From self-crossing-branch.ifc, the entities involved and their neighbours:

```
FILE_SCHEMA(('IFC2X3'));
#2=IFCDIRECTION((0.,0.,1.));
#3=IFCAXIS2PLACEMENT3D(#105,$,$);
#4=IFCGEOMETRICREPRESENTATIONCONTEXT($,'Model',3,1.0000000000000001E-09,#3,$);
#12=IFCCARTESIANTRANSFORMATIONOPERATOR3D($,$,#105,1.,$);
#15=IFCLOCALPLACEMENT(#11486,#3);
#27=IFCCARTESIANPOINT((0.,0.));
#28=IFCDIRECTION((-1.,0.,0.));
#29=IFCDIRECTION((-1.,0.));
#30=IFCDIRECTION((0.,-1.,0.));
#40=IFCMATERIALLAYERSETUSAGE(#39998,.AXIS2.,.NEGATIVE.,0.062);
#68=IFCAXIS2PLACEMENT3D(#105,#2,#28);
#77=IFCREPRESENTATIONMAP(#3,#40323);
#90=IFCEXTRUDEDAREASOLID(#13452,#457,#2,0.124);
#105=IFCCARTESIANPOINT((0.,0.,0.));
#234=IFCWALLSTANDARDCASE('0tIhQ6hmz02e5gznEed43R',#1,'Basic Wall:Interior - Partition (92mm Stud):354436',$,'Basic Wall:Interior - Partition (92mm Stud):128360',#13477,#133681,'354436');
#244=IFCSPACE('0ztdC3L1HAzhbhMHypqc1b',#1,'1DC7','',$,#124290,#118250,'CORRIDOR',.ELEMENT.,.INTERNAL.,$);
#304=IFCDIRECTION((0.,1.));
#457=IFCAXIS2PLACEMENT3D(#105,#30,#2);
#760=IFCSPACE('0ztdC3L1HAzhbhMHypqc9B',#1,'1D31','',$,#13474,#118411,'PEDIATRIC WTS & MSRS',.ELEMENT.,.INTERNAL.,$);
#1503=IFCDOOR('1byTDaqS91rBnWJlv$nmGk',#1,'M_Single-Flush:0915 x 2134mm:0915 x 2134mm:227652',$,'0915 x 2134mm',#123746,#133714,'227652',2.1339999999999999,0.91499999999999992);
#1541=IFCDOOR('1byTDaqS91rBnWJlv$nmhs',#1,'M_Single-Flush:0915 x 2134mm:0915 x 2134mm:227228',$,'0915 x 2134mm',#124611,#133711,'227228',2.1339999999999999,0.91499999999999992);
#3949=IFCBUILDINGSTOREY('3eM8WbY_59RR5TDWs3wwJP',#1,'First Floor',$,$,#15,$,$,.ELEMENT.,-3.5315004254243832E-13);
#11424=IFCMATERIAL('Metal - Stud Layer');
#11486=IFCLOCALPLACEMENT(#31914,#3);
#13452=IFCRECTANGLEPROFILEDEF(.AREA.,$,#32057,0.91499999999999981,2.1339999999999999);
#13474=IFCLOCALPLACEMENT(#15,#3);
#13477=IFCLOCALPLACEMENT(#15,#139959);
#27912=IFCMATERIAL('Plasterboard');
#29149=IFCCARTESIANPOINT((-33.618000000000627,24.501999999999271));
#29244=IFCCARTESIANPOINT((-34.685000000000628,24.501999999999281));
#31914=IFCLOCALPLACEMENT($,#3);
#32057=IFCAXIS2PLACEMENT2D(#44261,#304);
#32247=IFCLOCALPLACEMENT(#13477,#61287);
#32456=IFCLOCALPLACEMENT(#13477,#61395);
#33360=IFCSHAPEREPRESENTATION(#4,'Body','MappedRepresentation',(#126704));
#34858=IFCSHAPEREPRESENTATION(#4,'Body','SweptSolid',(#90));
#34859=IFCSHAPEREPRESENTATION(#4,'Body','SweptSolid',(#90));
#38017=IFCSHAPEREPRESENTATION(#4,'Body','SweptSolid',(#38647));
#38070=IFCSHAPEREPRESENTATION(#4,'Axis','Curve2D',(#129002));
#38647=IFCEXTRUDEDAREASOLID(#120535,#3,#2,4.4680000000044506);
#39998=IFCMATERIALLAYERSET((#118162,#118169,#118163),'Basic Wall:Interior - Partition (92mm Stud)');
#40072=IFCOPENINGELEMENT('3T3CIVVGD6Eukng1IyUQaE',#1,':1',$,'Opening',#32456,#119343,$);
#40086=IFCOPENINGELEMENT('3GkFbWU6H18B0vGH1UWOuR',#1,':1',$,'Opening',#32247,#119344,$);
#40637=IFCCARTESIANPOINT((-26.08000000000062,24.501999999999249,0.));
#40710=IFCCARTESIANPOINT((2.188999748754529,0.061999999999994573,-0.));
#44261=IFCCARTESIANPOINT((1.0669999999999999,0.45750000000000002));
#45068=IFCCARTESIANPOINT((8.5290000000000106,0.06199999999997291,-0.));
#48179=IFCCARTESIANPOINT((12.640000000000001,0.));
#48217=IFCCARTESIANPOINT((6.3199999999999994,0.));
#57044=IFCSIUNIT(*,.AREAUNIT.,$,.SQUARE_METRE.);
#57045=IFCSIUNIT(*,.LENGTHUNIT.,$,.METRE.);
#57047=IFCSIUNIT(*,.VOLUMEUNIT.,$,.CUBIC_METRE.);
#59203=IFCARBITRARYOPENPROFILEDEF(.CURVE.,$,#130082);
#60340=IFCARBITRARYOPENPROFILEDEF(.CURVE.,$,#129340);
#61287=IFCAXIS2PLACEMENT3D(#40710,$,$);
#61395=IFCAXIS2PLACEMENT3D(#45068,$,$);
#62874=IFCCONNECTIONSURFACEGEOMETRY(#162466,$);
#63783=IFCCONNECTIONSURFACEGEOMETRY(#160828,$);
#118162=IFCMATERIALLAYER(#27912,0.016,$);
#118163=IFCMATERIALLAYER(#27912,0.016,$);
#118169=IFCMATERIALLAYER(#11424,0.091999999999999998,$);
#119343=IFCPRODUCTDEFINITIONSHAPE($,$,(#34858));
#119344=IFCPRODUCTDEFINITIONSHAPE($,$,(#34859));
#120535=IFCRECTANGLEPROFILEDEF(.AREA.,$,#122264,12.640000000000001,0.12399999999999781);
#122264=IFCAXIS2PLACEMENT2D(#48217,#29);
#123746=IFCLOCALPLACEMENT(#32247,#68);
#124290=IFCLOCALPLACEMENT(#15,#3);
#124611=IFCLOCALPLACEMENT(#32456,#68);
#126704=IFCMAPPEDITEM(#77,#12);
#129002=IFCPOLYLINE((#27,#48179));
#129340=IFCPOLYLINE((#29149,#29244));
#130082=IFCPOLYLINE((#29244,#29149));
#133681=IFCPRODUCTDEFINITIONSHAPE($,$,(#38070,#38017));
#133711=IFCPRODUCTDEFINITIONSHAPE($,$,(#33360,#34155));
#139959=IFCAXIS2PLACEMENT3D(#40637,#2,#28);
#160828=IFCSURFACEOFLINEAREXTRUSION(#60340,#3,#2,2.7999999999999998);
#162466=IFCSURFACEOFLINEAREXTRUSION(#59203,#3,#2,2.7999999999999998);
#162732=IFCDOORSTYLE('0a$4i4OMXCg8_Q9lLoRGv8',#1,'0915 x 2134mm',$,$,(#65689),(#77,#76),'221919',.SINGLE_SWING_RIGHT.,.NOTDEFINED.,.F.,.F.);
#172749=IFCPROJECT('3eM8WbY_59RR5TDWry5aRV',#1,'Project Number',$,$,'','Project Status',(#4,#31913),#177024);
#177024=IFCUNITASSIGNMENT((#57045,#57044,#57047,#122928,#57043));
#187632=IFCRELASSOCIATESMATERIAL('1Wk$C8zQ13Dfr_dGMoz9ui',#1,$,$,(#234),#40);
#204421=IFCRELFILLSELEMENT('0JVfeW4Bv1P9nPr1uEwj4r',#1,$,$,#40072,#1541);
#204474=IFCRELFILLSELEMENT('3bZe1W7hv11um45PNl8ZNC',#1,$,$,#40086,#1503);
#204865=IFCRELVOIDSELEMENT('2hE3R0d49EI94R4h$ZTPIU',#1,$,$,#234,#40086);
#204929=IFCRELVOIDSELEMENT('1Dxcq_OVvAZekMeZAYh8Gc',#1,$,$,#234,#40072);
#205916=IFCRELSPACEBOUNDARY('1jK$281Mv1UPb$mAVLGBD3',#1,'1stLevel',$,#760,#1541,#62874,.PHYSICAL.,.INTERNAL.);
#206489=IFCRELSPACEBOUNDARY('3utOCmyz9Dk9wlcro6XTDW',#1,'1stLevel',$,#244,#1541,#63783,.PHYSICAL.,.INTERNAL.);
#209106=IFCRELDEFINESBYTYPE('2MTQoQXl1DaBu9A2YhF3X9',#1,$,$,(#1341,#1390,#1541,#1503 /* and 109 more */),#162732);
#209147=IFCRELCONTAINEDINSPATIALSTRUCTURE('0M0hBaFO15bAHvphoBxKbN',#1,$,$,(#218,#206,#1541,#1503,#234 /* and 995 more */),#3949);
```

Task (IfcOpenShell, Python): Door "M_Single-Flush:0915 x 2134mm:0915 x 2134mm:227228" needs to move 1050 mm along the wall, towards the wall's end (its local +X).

```python
import numpy as np
import ifcopenshell
import ifcopenshell.api.geometry
import ifcopenshell.util.placement

model = ifcopenshell.open("self-crossing-branch.ifc")

door = model.by_id(1541)
opening = door.FillsVoids[0].RelatingOpeningElement
wall = opening.VoidsElements[0].RelatingBuildingElement

wall_matrix = ifcopenshell.util.placement.get_local_placement(wall.ObjectPlacement)
shift = wall_matrix[:3, 0] * 1.05
before = ifcopenshell.util.placement.get_local_placement(door.ObjectPlacement)[:3, 3].copy()

# The door is placed relative to its opening, so it follows when the opening moves.
matrix = ifcopenshell.util.placement.get_local_placement(opening.ObjectPlacement)
matrix[:3, 3] += shift
ifcopenshell.api.geometry.edit_object_placement(
    model, product=opening, matrix=matrix, is_si=False, should_transform_children=True
)

# Space boundary surfaces are stored in each space's coordinates; move them too.
for rel in door.ProvidesBoundaries:
    if not rel.ConnectionGeometry:
        continue
    surface = rel.ConnectionGeometry.SurfaceOnRelatingElement
    space_matrix = ifcopenshell.util.placement.get_local_placement(rel.RelatingSpace.ObjectPlacement)
    point = np.array(surface.Position.Location.Coordinates) + space_matrix[:3, :3].T @ shift
    surface.Position = model.createIfcAxis2Placement3D(
        model.createIfcCartesianPoint(point.tolist()), surface.Position.Axis, surface.Position.RefDirection
    )

after = ifcopenshell.util.placement.get_local_placement(door.ObjectPlacement)[:3, 3]
print("door moved by", (after - before).round(3) + 0.0)

model.write("self-crossing-branch_edited.ifc")
```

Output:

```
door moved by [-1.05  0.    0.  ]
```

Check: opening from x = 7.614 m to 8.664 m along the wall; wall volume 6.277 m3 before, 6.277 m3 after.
